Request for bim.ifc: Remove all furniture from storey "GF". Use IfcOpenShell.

First a look at what the model holds.

```python
import ifcopenshell
import ifcopenshell.util.element

model = ifcopenshell.open("bim.ifc")
print(model.schema)
storey = next(s for s in model.by_type("IfcBuildingStorey") if s.Name == "GF")
furniture = [e for e in ifcopenshell.util.element.get_decomposition(storey) if e.is_a("IfcFurnishingElement")]
seen = {}
for e in furniture:
    element_type = ifcopenshell.util.element.get_type(e)
    name = element_type.Name if element_type not in (None, e) else None
    seen[name] = seen.get(name, 0) + 1
for name, count in sorted(seen.items(), key=str):
    print(count, "x", name)
```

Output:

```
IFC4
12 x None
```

```python
import ifcopenshell
import ifcopenshell.api.root
import ifcopenshell.util.element

model = ifcopenshell.open("bim.ifc")

storey = next(s for s in model.by_type("IfcBuildingStorey") if s.Name == "GF")
furniture = [e for e in ifcopenshell.util.element.get_decomposition(storey) if e.is_a("IfcFurnishingElement")]

for e in furniture:
    ifcopenshell.api.root.remove_product(model, product=e)
print(len(furniture), "removed")

model.write("bim_updated.ifc")
```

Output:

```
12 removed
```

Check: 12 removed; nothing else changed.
